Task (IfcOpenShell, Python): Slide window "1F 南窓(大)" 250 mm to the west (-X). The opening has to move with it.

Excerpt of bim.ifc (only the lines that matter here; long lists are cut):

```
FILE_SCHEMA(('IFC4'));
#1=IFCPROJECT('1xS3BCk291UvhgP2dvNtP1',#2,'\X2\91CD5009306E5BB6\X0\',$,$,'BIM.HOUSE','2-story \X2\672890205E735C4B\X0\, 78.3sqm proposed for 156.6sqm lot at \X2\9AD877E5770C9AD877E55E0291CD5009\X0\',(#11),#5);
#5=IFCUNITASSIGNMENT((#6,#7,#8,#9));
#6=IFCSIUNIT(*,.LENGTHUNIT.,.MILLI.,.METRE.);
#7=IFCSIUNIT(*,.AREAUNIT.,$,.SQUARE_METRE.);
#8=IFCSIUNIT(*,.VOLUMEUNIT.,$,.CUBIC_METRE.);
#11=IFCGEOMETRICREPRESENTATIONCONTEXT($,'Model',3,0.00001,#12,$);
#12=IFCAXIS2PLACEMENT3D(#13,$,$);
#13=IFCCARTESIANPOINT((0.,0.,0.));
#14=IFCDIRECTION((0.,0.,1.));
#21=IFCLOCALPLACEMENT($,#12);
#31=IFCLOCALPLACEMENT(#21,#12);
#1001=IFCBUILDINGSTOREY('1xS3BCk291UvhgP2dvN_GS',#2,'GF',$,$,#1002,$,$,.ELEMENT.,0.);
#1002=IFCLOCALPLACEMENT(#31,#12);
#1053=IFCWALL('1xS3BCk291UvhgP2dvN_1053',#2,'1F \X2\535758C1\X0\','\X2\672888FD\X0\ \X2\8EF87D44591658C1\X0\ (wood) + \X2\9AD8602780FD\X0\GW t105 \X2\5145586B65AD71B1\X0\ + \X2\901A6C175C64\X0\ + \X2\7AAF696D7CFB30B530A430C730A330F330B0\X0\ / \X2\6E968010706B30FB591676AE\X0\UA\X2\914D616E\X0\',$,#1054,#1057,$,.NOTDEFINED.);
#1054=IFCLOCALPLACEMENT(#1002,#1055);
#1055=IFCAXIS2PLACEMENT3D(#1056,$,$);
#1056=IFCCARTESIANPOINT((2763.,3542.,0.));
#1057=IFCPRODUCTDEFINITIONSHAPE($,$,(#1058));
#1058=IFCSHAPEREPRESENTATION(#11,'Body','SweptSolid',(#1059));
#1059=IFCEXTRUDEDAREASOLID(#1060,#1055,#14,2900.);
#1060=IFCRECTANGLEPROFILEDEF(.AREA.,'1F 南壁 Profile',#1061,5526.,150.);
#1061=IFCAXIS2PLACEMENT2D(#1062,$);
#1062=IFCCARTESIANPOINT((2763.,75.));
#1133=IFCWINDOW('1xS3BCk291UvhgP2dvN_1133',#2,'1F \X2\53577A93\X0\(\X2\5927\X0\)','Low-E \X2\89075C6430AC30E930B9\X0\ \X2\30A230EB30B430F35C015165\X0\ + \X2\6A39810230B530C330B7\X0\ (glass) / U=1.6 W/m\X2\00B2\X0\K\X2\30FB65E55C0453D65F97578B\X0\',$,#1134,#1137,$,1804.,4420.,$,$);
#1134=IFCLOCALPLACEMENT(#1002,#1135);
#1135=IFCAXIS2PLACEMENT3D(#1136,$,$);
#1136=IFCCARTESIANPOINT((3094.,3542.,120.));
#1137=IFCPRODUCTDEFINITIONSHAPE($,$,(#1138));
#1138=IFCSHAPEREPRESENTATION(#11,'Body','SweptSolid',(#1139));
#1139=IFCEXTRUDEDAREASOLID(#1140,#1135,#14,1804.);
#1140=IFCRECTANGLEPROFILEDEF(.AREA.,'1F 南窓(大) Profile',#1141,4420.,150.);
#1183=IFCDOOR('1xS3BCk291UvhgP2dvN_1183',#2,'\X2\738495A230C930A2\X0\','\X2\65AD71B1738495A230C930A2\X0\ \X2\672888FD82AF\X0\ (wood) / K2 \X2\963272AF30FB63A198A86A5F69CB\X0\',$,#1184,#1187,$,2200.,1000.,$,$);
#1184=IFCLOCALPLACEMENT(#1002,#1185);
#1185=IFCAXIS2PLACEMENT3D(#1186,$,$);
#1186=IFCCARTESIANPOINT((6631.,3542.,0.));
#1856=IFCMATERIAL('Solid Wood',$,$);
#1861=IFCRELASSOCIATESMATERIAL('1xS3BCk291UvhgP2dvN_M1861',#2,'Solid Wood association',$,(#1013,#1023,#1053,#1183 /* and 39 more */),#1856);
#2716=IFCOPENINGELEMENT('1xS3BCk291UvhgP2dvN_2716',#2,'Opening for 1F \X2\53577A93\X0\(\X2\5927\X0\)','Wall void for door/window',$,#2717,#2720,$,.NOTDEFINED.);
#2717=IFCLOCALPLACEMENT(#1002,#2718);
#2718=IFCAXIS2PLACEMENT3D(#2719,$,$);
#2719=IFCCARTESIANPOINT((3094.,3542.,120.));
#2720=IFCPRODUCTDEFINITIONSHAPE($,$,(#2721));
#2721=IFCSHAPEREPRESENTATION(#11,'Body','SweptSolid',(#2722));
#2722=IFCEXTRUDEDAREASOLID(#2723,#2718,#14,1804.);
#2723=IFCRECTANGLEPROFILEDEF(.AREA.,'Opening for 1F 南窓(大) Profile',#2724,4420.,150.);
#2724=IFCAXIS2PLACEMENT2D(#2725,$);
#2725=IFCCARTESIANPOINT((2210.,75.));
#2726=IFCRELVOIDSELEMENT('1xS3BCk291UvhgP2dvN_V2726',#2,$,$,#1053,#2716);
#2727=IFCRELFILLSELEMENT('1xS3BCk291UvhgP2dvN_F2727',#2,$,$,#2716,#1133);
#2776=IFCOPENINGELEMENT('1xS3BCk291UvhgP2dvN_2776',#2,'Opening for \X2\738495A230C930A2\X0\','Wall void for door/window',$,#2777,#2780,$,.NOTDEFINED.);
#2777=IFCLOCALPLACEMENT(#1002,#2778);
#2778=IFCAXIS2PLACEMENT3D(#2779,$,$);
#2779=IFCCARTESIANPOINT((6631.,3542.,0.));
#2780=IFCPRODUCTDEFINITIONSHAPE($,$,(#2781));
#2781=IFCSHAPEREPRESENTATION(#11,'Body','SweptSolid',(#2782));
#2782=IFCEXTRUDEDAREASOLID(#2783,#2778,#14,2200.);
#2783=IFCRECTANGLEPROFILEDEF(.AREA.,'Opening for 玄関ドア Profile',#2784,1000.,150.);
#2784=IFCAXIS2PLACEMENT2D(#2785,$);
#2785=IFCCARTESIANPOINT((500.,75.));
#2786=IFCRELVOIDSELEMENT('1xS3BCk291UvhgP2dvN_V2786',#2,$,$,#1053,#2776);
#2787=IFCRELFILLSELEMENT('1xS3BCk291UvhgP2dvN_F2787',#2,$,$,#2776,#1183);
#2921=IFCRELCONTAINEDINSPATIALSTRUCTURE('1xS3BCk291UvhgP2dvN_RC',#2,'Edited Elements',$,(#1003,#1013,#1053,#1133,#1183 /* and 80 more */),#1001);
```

```python
import ifcopenshell
import ifcopenshell.api.geometry
import ifcopenshell.util.placement
import ifcopenshell.util.unit

model = ifcopenshell.open("bim.ifc")
unit_scale = ifcopenshell.util.unit.calculate_unit_scale(model)

window = model.by_id(1133)
opening = window.FillsVoids[0].RelatingOpeningElement
wall = opening.VoidsElements[0].RelatingBuildingElement

wall_matrix = ifcopenshell.util.placement.get_local_placement(wall.ObjectPlacement)
shift = wall_matrix[:3, 0] * -0.25 / unit_scale
before = ifcopenshell.util.placement.get_local_placement(window.ObjectPlacement)[:3, 3].copy()

# The window is not placed relative to its opening, so move both.
for product in (opening, window):
    matrix = ifcopenshell.util.placement.get_local_placement(product.ObjectPlacement)
    matrix[:3, 3] += shift
    ifcopenshell.api.geometry.edit_object_placement(model, product=product, matrix=matrix, is_si=False)

after = ifcopenshell.util.placement.get_local_placement(window.ObjectPlacement)[:3, 3]
print("window moved by", (after - before).round(3) + 0.0)

model.write("bim_updated.ifc")
```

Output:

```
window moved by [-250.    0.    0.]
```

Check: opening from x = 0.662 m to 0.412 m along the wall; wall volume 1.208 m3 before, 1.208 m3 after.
